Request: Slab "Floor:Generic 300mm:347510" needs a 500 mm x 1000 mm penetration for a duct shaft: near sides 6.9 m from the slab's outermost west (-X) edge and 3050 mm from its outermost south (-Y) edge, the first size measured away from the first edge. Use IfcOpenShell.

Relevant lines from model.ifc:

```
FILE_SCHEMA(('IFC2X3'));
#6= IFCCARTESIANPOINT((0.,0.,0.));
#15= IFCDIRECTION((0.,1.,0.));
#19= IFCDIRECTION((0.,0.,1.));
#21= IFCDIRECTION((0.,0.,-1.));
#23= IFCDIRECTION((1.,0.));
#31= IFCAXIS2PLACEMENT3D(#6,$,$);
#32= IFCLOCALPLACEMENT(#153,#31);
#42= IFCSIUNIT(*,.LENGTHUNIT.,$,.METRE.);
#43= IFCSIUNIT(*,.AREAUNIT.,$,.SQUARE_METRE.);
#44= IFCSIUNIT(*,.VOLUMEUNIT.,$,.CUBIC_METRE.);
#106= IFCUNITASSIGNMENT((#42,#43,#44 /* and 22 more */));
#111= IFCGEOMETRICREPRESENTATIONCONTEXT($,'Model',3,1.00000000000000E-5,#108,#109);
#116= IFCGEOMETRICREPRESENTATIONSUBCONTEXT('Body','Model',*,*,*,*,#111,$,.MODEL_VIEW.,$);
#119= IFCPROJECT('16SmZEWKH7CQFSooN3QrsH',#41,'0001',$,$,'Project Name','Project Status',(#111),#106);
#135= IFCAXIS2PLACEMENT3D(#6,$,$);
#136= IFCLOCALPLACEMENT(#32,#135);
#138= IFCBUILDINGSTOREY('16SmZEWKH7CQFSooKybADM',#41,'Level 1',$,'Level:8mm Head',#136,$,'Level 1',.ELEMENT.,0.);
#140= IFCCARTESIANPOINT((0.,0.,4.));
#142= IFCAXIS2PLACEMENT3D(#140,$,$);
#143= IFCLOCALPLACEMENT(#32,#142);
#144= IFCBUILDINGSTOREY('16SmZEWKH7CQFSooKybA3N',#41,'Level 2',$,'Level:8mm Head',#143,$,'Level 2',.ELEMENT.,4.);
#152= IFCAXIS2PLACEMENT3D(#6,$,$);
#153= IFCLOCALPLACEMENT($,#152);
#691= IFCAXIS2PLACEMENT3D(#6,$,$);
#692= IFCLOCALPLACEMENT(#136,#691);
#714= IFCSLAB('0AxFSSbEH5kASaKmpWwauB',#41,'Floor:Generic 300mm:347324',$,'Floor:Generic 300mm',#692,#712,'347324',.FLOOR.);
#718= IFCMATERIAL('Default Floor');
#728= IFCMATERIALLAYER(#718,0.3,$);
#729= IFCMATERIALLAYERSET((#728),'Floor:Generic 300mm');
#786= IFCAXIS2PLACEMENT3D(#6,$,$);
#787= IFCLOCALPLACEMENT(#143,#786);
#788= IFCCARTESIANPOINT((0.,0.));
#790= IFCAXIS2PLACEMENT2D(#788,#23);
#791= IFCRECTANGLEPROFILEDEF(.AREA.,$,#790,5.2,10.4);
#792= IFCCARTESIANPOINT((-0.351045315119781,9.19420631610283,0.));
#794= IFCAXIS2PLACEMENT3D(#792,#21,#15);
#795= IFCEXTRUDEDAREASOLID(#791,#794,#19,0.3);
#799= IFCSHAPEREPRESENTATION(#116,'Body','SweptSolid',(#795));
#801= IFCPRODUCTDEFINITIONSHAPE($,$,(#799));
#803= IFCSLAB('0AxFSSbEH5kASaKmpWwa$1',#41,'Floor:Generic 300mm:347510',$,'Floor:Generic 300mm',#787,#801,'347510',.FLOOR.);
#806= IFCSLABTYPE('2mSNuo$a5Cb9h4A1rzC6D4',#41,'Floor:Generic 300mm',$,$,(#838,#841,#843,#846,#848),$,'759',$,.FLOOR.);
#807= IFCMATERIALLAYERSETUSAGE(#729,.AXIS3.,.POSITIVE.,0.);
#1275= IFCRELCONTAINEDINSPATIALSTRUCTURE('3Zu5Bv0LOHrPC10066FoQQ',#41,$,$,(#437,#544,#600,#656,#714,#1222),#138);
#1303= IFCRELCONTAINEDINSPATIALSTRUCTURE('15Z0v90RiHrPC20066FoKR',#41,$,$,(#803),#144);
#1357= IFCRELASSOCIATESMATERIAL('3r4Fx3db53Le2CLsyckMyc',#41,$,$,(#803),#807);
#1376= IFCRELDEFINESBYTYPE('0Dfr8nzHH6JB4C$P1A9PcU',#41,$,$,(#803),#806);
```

```python
import numpy as np
import ifcopenshell
import ifcopenshell.api.feature
import ifcopenshell.api.geometry
import ifcopenshell.api.root
import ifcopenshell.geom
import ifcopenshell.util.placement
import ifcopenshell.util.representation
import ifcopenshell.util.shape
import ifcopenshell.util.unit

model = ifcopenshell.open("model.ifc")
unit_scale = ifcopenshell.util.unit.calculate_unit_scale(model)
settings = ifcopenshell.geom.settings()


def volume(element):
    """Net volume in cubic metres, openings subtracted."""
    shape = ifcopenshell.geom.create_shape(settings, element)
    return ifcopenshell.util.shape.get_volume(shape.geometry)


slab = model.by_guid("0AxFSSbEH5kASaKmpWwa$1")
before = volume(slab)

# Extent in the slab's own axes, in metres. The edges named are its -X and -Y sides.
slab_shape = ifcopenshell.geom.create_shape(settings, slab)
vertices = ifcopenshell.util.shape.get_vertices(slab_shape.geometry)
x_min, y_min, bottom = vertices.min(axis=0)
top = vertices[:, 2].max()

opening = ifcopenshell.api.root.create_entity(model, ifc_class="IfcOpeningElement", name="Duct shaft opening")
context = ifcopenshell.util.representation.get_context(model, "Model", "Body", "MODEL_VIEW")
width, depth = 0.5, 1
outline = [(0.0, 0.0), (width, 0.0), (width, depth), (0.0, depth), (0.0, 0.0)]
# Overshoot both faces by 50 mm so the cut is clean.
shape = ifcopenshell.api.geometry.add_slab_representation(
    model, context=context, depth=top - bottom + 0.1, polyline=outline
)
ifcopenshell.api.geometry.assign_representation(model, product=opening, representation=shape)

matrix = ifcopenshell.util.placement.get_local_placement(slab.ObjectPlacement)
matrix[:, 3] = matrix @ np.append(np.array([x_min + 6.9, y_min + 3.05, bottom - 0.05]) / unit_scale, 1.0)
ifcopenshell.api.geometry.edit_object_placement(model, product=opening, matrix=matrix, is_si=False)
ifcopenshell.api.feature.add_feature(model, feature=opening, element=slab)

after = volume(slab)

print(f"slab volume {before:.3f} -> {after:.3f} m3")

model.write("model_rev.ifc")
```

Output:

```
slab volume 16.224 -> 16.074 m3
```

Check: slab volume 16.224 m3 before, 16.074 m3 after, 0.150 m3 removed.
